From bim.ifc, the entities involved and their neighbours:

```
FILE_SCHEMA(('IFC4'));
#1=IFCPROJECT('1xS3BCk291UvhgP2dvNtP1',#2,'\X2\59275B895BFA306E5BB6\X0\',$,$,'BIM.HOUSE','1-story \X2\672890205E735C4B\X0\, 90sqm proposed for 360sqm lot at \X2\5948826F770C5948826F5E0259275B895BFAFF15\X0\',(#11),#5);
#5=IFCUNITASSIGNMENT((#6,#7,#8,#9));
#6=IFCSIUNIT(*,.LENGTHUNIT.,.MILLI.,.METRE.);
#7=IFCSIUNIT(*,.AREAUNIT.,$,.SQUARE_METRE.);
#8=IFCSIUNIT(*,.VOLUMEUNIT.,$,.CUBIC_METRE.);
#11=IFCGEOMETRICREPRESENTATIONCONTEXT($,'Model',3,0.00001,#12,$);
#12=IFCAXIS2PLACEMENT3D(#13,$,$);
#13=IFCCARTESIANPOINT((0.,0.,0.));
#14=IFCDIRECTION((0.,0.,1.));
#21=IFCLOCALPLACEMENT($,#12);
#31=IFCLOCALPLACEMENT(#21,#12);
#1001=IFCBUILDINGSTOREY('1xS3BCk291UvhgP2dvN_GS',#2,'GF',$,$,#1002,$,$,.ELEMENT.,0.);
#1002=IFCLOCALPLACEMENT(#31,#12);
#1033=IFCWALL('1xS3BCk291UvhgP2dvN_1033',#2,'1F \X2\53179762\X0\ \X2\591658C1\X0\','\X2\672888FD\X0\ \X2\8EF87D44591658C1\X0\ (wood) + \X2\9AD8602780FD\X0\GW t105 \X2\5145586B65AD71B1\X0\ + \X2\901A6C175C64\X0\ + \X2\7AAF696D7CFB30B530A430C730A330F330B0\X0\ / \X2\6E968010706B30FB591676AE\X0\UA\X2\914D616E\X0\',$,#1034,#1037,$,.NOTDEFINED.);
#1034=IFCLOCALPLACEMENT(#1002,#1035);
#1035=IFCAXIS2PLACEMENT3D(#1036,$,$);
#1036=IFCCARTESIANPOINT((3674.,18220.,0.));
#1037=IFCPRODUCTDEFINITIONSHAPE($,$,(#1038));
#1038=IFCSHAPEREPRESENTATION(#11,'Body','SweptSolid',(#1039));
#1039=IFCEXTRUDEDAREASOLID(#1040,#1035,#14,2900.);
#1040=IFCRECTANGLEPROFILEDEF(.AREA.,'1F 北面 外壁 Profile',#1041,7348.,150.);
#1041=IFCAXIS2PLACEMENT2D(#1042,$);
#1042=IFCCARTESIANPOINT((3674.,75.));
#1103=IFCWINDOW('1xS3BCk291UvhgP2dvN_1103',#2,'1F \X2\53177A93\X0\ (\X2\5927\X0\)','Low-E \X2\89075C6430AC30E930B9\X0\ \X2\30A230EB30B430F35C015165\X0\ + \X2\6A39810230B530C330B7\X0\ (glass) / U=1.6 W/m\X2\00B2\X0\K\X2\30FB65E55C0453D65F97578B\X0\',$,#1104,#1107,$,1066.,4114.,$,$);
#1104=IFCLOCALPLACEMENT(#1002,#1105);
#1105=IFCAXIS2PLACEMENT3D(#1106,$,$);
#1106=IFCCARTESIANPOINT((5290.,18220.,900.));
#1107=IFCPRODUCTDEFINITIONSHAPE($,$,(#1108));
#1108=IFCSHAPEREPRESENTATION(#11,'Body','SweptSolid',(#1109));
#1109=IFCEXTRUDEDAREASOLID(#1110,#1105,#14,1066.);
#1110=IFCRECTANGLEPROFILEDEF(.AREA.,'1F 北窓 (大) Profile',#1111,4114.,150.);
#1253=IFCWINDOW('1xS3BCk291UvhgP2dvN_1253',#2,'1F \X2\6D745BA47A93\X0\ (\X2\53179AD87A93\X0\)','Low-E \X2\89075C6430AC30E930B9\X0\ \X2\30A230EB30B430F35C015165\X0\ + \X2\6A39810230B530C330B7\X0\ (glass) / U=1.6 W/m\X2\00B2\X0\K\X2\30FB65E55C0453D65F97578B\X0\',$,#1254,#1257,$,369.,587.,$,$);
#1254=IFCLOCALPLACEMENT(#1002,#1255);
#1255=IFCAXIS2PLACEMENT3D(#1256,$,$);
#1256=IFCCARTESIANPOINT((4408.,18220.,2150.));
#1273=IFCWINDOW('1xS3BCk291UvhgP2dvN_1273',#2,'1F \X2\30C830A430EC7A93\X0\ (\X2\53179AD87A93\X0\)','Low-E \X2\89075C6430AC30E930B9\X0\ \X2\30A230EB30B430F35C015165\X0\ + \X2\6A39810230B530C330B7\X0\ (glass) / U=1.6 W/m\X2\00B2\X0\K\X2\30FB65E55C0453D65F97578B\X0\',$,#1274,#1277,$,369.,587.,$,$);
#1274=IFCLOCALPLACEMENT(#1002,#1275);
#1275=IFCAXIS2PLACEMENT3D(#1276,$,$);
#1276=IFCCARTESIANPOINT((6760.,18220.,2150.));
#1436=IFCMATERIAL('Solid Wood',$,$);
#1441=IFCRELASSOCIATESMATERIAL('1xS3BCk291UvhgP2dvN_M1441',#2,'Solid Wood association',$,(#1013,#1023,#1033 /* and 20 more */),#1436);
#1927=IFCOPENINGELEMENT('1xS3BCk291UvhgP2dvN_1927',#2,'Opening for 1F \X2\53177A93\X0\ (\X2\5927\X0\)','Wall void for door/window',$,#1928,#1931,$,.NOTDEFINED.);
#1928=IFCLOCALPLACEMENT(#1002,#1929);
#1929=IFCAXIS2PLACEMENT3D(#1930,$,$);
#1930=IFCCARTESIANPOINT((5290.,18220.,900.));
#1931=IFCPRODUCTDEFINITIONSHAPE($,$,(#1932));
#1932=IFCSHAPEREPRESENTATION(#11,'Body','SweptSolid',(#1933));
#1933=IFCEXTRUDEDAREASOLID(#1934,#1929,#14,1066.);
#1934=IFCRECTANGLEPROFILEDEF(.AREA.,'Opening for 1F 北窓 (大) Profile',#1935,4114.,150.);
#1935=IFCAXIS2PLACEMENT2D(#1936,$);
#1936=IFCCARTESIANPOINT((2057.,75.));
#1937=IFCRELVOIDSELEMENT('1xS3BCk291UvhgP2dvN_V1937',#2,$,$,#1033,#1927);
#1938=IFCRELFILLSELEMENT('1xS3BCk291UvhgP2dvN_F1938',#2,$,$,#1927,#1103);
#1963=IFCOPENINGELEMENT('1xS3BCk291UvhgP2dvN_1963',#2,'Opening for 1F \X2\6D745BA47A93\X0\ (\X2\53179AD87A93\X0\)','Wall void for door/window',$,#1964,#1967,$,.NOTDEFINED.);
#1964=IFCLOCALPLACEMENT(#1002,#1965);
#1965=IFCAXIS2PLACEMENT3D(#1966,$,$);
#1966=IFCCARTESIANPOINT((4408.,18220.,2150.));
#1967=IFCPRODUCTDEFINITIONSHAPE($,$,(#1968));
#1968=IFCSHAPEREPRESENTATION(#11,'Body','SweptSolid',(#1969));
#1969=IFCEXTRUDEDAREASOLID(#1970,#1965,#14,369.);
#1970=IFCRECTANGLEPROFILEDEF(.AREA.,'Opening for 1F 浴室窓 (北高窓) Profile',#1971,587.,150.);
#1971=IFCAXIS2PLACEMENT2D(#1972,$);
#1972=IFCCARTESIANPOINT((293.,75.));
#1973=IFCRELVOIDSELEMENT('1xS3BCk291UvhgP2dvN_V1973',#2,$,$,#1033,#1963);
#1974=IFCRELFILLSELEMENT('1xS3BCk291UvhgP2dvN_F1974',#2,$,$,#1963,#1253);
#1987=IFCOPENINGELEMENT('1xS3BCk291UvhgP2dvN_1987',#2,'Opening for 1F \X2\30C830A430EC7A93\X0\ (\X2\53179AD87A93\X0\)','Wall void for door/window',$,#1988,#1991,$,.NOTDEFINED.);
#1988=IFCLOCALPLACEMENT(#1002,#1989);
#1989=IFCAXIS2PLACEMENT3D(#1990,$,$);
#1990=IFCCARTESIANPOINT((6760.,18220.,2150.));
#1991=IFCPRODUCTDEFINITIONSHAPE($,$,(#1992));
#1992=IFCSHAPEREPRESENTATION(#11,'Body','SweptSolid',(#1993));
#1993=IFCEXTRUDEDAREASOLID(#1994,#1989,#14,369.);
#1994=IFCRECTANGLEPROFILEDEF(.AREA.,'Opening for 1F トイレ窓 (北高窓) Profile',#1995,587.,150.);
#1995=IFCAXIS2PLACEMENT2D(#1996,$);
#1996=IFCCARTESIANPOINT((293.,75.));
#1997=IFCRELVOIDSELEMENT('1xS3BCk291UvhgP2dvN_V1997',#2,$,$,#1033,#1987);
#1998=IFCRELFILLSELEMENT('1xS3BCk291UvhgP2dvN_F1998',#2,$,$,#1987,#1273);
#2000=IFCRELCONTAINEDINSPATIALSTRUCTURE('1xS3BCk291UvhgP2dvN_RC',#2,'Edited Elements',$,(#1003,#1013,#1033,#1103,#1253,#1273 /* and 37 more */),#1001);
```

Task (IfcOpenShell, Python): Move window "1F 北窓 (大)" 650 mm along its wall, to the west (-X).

```python
import ifcopenshell
import ifcopenshell.api.geometry
import ifcopenshell.util.placement
import ifcopenshell.util.unit

model = ifcopenshell.open("bim.ifc")
unit_scale = ifcopenshell.util.unit.calculate_unit_scale(model)

window = model.by_guid("1xS3BCk291UvhgP2dvN_1103")
opening = window.FillsVoids[0].RelatingOpeningElement
wall = opening.VoidsElements[0].RelatingBuildingElement

wall_matrix = ifcopenshell.util.placement.get_local_placement(wall.ObjectPlacement)
shift = wall_matrix[:3, 0] * -0.65 / unit_scale
before = ifcopenshell.util.placement.get_local_placement(window.ObjectPlacement)[:3, 3].copy()

# The window is not placed relative to its opening, so move both.
for product in (opening, window):
    matrix = ifcopenshell.util.placement.get_local_placement(product.ObjectPlacement)
    matrix[:3, 3] += shift
    ifcopenshell.api.geometry.edit_object_placement(model, product=product, matrix=matrix, is_si=False)

after = ifcopenshell.util.placement.get_local_placement(window.ObjectPlacement)[:3, 3]
print("window moved by", (after - before).round(3) + 0.0)

model.write("bim_v2.ifc")
```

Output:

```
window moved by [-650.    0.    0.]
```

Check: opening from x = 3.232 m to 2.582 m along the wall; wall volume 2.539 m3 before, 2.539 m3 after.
